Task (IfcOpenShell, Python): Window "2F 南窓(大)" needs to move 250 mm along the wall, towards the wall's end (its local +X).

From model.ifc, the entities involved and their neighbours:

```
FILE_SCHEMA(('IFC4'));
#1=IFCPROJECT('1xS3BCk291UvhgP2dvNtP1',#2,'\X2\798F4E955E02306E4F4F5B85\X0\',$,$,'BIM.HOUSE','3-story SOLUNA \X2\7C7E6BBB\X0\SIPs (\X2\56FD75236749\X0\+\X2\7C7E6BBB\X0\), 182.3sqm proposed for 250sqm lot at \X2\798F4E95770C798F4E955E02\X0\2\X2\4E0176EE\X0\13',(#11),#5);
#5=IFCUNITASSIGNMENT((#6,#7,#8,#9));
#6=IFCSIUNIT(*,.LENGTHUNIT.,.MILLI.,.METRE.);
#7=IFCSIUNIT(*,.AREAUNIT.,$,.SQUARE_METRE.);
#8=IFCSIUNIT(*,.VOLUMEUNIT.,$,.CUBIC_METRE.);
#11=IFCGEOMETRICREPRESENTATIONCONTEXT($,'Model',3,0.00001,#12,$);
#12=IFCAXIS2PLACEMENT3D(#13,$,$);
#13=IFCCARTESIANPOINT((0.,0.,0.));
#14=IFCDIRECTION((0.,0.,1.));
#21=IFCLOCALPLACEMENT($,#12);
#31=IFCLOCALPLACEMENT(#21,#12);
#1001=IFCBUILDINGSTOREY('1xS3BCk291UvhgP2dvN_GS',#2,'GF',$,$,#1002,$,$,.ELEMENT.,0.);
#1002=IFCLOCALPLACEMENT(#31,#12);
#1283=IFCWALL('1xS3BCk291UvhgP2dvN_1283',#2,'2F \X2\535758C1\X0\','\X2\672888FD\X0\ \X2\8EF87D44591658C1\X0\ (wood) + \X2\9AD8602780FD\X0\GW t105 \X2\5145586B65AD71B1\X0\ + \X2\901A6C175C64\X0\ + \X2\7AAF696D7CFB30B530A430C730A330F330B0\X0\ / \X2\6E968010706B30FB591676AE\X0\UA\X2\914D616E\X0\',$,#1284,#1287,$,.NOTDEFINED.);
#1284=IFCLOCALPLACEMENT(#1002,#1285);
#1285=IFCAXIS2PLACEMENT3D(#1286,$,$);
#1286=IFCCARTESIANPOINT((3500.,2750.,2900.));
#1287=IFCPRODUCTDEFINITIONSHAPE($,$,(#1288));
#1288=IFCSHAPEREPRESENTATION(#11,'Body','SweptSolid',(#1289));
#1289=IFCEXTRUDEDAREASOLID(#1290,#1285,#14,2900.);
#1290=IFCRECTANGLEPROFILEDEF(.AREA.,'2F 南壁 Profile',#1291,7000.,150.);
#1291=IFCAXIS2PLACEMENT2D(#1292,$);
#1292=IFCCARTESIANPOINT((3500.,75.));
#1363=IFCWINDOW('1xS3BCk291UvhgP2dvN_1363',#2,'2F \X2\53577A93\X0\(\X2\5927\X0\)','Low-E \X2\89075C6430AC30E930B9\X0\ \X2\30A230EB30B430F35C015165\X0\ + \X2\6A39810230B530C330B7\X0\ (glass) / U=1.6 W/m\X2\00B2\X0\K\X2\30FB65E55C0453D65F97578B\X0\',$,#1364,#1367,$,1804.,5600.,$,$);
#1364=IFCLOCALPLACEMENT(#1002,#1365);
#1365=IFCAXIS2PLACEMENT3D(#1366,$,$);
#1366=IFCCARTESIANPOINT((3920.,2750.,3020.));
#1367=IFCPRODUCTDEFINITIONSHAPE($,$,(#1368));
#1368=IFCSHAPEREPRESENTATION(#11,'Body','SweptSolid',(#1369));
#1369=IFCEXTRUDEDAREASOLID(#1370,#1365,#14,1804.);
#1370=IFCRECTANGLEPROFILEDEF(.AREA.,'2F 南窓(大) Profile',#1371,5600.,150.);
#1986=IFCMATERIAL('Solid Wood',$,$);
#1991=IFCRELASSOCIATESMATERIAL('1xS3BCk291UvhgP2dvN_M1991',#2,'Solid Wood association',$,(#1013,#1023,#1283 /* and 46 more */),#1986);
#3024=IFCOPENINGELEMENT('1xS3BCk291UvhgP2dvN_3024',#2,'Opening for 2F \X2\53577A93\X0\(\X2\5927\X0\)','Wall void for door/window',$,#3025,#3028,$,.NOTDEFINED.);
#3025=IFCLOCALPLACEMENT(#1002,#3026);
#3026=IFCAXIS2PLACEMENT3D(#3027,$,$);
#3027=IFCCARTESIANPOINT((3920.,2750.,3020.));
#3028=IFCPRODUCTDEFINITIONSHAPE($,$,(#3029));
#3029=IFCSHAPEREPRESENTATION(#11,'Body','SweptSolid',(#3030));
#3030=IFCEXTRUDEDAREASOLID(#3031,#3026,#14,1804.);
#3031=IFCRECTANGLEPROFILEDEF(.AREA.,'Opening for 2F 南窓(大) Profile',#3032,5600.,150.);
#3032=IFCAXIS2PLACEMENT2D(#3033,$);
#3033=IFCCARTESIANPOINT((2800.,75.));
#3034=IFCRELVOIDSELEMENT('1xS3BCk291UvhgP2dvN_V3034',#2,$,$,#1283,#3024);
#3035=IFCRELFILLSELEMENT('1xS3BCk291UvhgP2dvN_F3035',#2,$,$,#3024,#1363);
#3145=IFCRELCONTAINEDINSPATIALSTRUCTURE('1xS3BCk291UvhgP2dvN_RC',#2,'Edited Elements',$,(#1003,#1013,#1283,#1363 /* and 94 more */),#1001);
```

```python
import ifcopenshell
import ifcopenshell.api.geometry
import ifcopenshell.util.placement

model = ifcopenshell.open("model.ifc")

window = model.by_guid("1xS3BCk291UvhgP2dvN_1363")
opening = window.FillsVoids[0].RelatingOpeningElement
wall = opening.VoidsElements[0].RelatingBuildingElement

wall_matrix = ifcopenshell.util.placement.get_local_placement(wall.ObjectPlacement)
shift = wall_matrix[:3, 0] * 250.0
before = ifcopenshell.util.placement.get_local_placement(window.ObjectPlacement)[:3, 3].copy()

# The window is not placed relative to its opening, so move both.
for product in (opening, window):
    matrix = ifcopenshell.util.placement.get_local_placement(product.ObjectPlacement)
    matrix[:3, 3] += shift
    ifcopenshell.api.geometry.edit_object_placement(model, product=product, matrix=matrix, is_si=False)

after = ifcopenshell.util.placement.get_local_placement(window.ObjectPlacement)[:3, 3]
print("window moved by", (after - before).round(3) + 0.0)

model.write("model_v2.ifc")
```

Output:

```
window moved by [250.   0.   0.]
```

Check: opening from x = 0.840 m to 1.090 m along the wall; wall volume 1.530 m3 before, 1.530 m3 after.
